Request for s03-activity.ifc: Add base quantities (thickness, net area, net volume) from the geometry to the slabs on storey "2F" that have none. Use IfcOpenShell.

First a look at what the model holds.

```python
import ifcopenshell
import ifcopenshell.util.element
import ifcopenshell.util.unit

model = ifcopenshell.open("s03-activity.ifc")
print(model.schema)
for unit_type in ("LENGTHUNIT", "AREAUNIT", "VOLUMEUNIT"):
    print(unit_type, ifcopenshell.util.unit.calculate_unit_scale(model, unit_type))
storey = next(s for s in model.by_type("IfcBuildingStorey") if s.Name == "2F")
slabs = [e for e in ifcopenshell.util.element.get_decomposition(storey) if e.is_a("IfcSlab")]
for e in sorted(slabs, key=lambda e: e.id()):
    print(e.id(), e.is_a(), e.Name, list(ifcopenshell.util.element.get_psets(e, qtos_only=True)), sep=" | ")
```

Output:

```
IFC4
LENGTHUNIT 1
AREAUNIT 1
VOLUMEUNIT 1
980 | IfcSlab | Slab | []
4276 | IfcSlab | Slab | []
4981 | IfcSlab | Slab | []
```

```python
import ifcopenshell
import ifcopenshell.api.pset
import ifcopenshell.geom
import ifcopenshell.util.element
import ifcopenshell.util.shape
import ifcopenshell.util.unit

model = ifcopenshell.open("s03-activity.ifc")
unit_scale = ifcopenshell.util.unit.calculate_unit_scale(model)
area_scale = ifcopenshell.util.unit.calculate_unit_scale(model, "AREAUNIT")
volume_scale = ifcopenshell.util.unit.calculate_unit_scale(model, "VOLUMEUNIT")
settings = ifcopenshell.geom.settings()

storey = next(s for s in model.by_type("IfcBuildingStorey") if s.Name == "2F")
slabs = [e for e in ifcopenshell.util.element.get_decomposition(storey) if e.is_a("IfcSlab")]

for e in sorted(slabs, key=lambda e: e.id()):
    if ifcopenshell.util.element.get_psets(e, qtos_only=True, should_inherit=False):
        continue
    # Geometry comes back in metres, in the element's own axes.
    shape = ifcopenshell.geom.create_shape(settings, e)
    values = {
        "Width": ifcopenshell.util.shape.get_z(shape.geometry) / unit_scale,
        "NetArea": ifcopenshell.util.shape.get_footprint_area(shape.geometry) / area_scale,
        "NetVolume": ifcopenshell.util.shape.get_volume(shape.geometry) / volume_scale,
    }
    qto = ifcopenshell.api.pset.add_qto(model, product=e, name="Qto_SlabBaseQuantities")
    ifcopenshell.api.pset.edit_qto(model, qto=qto, properties=values)
    print(e.id(), {k: round(v, 3) for k, v in values.items()})

model.write("s03-activity_rev.ifc")
```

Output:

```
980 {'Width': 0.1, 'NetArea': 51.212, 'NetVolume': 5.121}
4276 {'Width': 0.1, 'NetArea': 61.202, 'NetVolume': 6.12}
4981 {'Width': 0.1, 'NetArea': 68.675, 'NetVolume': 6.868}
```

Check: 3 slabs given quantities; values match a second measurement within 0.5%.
